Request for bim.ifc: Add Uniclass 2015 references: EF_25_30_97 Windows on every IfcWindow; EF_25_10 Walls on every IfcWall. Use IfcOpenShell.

First a look at what the model holds.

```python
import ifcopenshell

model = ifcopenshell.open("bim.ifc")
print(model.schema)
print("classifications:", [c.Name for c in model.by_type("IfcClassification")])
for ifc_class in ("IfcDoor", "IfcRoof", "IfcStair", "IfcWall", "IfcWindow"):
    print(ifc_class, len(model.by_type(ifc_class)))
```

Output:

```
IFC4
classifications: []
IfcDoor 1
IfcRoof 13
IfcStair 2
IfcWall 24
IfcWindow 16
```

```python
import ifcopenshell
import ifcopenshell.api.classification

model = ifcopenshell.open("bim.ifc")

system = ifcopenshell.api.classification.add_classification(model, classification="Uniclass 2015")

codes = {
    "IfcWindow": ("EF_25_30_97", "Windows"),
    "IfcWall": ("EF_25_10", "Walls"),
}
for ifc_class, (code, name) in codes.items():
    products = model.by_type(ifc_class)
    ifcopenshell.api.classification.add_reference(
        model, products=products, classification=system, identification=code, name=name
    )
    print(code, len(products))

model.write("bim_updated.ifc")
```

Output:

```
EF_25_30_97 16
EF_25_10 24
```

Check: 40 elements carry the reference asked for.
